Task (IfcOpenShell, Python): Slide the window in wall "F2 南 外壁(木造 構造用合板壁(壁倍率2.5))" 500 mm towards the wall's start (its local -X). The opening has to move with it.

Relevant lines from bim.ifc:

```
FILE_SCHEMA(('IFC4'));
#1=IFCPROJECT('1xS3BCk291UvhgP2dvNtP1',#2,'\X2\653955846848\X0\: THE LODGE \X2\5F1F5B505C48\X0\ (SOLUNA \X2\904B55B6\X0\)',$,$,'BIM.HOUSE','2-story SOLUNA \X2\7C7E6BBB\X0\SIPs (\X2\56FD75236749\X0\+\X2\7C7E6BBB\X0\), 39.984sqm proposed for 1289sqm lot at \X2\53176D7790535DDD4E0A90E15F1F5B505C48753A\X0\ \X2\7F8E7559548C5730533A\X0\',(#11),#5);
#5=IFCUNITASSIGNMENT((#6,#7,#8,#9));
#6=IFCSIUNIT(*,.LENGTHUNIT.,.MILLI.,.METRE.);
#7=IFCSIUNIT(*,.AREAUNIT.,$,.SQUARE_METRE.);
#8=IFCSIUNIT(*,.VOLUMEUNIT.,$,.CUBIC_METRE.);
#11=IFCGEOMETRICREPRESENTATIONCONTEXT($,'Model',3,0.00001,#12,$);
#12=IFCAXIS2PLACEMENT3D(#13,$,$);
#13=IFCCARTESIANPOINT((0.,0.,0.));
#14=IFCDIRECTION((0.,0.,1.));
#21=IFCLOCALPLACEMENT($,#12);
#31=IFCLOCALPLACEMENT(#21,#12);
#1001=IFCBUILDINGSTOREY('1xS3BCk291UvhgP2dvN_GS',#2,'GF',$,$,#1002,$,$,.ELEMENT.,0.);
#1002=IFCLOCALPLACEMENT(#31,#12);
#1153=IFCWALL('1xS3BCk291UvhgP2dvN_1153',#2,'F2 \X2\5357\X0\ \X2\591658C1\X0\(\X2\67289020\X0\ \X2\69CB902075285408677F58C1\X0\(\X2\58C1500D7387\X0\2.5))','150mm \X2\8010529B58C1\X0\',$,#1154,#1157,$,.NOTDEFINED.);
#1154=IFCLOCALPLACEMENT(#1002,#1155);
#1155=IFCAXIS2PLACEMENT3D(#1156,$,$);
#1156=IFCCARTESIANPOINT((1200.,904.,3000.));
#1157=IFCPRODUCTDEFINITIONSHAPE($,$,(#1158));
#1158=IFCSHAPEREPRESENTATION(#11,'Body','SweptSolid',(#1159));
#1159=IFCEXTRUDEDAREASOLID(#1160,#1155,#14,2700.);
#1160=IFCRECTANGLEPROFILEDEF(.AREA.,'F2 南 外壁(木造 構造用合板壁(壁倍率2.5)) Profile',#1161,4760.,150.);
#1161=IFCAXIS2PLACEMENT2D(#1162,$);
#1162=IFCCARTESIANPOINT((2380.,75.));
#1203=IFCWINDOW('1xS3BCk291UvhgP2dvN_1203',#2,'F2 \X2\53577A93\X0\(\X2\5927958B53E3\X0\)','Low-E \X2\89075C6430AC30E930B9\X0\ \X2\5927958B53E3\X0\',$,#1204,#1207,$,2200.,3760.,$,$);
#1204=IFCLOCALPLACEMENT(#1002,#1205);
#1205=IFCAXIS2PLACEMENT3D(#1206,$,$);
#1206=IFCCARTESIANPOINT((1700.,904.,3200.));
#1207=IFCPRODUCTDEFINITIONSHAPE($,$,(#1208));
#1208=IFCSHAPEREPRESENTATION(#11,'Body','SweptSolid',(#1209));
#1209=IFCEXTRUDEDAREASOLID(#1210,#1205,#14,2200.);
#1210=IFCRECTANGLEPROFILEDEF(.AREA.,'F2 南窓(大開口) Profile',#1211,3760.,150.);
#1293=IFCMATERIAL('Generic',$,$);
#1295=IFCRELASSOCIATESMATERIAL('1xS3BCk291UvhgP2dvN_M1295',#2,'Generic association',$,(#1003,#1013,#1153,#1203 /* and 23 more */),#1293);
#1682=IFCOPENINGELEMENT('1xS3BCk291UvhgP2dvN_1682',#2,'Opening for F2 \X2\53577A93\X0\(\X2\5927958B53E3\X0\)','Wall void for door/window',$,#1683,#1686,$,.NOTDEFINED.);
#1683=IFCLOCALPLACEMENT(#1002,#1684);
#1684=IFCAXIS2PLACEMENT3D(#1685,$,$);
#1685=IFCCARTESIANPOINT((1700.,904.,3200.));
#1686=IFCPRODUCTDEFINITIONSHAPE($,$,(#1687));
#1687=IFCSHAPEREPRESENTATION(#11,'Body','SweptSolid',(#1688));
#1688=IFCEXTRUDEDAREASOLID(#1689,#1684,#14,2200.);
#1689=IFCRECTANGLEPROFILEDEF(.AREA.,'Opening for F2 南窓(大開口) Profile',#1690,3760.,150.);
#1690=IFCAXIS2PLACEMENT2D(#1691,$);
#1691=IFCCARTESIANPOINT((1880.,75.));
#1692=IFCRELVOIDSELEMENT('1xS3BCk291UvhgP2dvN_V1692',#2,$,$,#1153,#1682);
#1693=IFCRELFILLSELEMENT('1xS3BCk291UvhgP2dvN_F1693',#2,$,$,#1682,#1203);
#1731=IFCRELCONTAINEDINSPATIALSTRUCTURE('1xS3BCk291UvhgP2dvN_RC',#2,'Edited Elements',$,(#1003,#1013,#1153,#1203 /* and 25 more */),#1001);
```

```python
import ifcopenshell
import ifcopenshell.api.geometry
import ifcopenshell.util.placement
import ifcopenshell.util.unit

model = ifcopenshell.open("bim.ifc")
unit_scale = ifcopenshell.util.unit.calculate_unit_scale(model)

window = model.by_guid("1xS3BCk291UvhgP2dvN_1203")
opening = window.FillsVoids[0].RelatingOpeningElement
wall = opening.VoidsElements[0].RelatingBuildingElement

wall_matrix = ifcopenshell.util.placement.get_local_placement(wall.ObjectPlacement)
shift = wall_matrix[:3, 0] * -0.5 / unit_scale
before = ifcopenshell.util.placement.get_local_placement(window.ObjectPlacement)[:3, 3].copy()

# The window is not placed relative to its opening, so move both.
for product in (opening, window):
    matrix = ifcopenshell.util.placement.get_local_placement(product.ObjectPlacement)
    matrix[:3, 3] += shift
    ifcopenshell.api.geometry.edit_object_placement(model, product=product, matrix=matrix, is_si=False)

after = ifcopenshell.util.placement.get_local_placement(window.ObjectPlacement)[:3, 3]
print("window moved by", (after - before).round(3) + 0.0)

model.write("bim-out.ifc")
```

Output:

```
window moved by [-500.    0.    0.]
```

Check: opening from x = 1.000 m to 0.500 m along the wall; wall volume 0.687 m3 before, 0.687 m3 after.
